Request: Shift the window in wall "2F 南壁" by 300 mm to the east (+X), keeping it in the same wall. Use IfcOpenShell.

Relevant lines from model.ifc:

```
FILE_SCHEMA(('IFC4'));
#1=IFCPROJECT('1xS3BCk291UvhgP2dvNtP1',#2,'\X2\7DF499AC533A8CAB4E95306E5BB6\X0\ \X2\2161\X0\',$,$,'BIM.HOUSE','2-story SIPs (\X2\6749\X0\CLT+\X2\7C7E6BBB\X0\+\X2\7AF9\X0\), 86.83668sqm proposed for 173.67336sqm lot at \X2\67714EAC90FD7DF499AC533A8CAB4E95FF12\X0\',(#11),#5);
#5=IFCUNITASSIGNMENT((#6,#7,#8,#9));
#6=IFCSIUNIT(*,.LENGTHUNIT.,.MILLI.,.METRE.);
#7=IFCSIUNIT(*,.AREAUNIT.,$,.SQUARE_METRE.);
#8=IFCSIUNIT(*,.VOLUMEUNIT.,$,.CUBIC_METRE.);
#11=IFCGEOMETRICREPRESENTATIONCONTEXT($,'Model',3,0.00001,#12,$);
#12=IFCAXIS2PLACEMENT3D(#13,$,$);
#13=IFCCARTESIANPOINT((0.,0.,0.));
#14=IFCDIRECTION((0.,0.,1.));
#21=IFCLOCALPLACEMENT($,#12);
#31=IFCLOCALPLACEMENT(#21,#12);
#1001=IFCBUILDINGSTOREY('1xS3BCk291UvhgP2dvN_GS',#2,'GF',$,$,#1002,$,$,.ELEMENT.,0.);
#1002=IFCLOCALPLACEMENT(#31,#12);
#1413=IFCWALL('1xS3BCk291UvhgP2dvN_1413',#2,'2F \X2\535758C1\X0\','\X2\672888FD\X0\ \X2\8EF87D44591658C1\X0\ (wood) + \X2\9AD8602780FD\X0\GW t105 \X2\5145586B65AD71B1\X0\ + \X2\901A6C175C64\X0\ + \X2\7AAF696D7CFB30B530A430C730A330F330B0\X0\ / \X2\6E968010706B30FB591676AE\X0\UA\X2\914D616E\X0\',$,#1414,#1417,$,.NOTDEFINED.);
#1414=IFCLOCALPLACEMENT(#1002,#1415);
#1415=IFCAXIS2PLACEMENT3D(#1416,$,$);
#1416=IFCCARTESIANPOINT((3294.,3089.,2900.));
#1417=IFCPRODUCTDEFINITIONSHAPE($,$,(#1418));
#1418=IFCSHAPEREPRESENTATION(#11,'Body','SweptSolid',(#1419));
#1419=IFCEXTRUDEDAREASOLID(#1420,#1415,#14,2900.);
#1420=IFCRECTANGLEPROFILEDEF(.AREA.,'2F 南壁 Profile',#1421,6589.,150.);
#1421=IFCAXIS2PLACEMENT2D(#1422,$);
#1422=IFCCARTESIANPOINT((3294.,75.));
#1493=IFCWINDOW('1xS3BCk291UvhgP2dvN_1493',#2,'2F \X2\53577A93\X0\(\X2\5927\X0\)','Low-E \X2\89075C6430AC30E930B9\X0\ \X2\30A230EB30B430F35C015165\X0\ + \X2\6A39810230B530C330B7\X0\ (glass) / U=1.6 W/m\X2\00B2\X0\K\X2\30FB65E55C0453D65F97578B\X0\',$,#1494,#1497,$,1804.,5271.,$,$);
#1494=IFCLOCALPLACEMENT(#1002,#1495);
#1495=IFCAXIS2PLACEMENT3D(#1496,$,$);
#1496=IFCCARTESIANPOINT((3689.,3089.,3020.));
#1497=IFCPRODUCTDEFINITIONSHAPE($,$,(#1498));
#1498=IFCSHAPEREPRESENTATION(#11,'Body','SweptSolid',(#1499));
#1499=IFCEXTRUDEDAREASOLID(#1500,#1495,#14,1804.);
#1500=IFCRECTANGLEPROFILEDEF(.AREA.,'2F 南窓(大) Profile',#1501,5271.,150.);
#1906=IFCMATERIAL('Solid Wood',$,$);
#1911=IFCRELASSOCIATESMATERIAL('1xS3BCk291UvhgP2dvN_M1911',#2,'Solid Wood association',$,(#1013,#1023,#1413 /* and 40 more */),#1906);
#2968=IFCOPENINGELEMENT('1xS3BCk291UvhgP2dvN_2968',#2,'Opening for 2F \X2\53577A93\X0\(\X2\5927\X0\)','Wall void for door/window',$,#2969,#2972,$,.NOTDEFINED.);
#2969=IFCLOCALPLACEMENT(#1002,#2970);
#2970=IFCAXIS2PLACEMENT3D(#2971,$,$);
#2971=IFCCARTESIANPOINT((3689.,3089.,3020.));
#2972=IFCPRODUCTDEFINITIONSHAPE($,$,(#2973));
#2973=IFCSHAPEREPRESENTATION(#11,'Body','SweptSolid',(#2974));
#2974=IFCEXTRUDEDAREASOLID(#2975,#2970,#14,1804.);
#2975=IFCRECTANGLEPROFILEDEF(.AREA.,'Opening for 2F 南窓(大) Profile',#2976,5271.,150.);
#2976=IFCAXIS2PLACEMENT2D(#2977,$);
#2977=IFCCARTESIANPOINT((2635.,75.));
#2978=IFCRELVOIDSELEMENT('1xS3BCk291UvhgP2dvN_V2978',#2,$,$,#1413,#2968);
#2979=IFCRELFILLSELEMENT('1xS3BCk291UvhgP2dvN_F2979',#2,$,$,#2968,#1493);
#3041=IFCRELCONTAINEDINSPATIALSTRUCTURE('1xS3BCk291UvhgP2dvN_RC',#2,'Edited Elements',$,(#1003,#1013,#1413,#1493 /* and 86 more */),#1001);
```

```python
import ifcopenshell
import ifcopenshell.api.geometry
import ifcopenshell.util.placement
import ifcopenshell.util.unit

model = ifcopenshell.open("model.ifc")
unit_scale = ifcopenshell.util.unit.calculate_unit_scale(model)

window = model.by_guid("1xS3BCk291UvhgP2dvN_1493")
opening = window.FillsVoids[0].RelatingOpeningElement
wall = opening.VoidsElements[0].RelatingBuildingElement

wall_matrix = ifcopenshell.util.placement.get_local_placement(wall.ObjectPlacement)
shift = wall_matrix[:3, 0] * 0.3 / unit_scale
before = ifcopenshell.util.placement.get_local_placement(window.ObjectPlacement)[:3, 3].copy()

# The window is not placed relative to its opening, so move both.
for product in (opening, window):
    matrix = ifcopenshell.util.placement.get_local_placement(product.ObjectPlacement)
    matrix[:3, 3] += shift
    ifcopenshell.api.geometry.edit_object_placement(model, product=product, matrix=matrix, is_si=False)

after = ifcopenshell.util.placement.get_local_placement(window.ObjectPlacement)[:3, 3]
print("window moved by", (after - before).round(3) + 0.0)

model.write("model_edited.ifc")
```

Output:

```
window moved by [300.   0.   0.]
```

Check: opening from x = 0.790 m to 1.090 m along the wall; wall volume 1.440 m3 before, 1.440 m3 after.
